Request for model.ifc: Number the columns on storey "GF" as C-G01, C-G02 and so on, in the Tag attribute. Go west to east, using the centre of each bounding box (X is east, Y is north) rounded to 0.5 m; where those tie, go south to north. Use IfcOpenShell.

First a look at what the model holds.

```python
import ifcopenshell
import ifcopenshell.util.element
import ifcopenshell.util.placement

model = ifcopenshell.open("model.ifc")
print(model.schema)
storey = next(s for s in model.by_type("IfcBuildingStorey") if s.Name == "GF")
columns = [e for e in ifcopenshell.util.element.get_decomposition(storey) if e.is_a("IfcColumn")]
for e in sorted(columns, key=lambda e: e.id()):
    origin = ifcopenshell.util.placement.get_local_placement(e.ObjectPlacement)[:3, 3]
    print(e.id(), e.Tag, e.Name, origin.round(2) + 0.0, sep=" | ")
```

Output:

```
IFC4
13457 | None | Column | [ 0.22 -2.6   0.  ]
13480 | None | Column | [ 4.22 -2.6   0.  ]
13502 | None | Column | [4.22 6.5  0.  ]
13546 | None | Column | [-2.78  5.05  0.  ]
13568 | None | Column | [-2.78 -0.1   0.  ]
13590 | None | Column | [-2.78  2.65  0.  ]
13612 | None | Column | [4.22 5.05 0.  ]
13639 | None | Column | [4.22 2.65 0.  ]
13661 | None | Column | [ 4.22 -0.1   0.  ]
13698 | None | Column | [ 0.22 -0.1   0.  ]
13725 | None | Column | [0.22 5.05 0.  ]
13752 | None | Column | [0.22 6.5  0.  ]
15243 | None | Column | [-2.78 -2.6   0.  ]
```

```python
import ifcopenshell
import ifcopenshell.geom
import ifcopenshell.util.element
import ifcopenshell.util.shape

model = ifcopenshell.open("model.ifc")
settings = ifcopenshell.geom.settings()
settings.set("use-world-coords", True)


def centre(element):
    shape = ifcopenshell.geom.create_shape(settings, element)
    return ifcopenshell.util.shape.get_bbox_centroid(shape.geometry)


storey = next(s for s in model.by_type("IfcBuildingStorey") if s.Name == "GF")
columns = [e for e in ifcopenshell.util.element.get_decomposition(storey) if e.is_a("IfcColumn")]

# Insertion points can sit at a corner or the storey origin, so sort by the geometry (in metres).
centres = {e: centre(e) for e in columns}
columns.sort(key=lambda e: (round(centres[e][0] / 0.5), centres[e][1]))

for i, e in enumerate(columns, start=1):
    number = f"C-G{i:02d}"
    e.Tag = number
    print(e.id(), number)

model.write("model_edited.ifc")
```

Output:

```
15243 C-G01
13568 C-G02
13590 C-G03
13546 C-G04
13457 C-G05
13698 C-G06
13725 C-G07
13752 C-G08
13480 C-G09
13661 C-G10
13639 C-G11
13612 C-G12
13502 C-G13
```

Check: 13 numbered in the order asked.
